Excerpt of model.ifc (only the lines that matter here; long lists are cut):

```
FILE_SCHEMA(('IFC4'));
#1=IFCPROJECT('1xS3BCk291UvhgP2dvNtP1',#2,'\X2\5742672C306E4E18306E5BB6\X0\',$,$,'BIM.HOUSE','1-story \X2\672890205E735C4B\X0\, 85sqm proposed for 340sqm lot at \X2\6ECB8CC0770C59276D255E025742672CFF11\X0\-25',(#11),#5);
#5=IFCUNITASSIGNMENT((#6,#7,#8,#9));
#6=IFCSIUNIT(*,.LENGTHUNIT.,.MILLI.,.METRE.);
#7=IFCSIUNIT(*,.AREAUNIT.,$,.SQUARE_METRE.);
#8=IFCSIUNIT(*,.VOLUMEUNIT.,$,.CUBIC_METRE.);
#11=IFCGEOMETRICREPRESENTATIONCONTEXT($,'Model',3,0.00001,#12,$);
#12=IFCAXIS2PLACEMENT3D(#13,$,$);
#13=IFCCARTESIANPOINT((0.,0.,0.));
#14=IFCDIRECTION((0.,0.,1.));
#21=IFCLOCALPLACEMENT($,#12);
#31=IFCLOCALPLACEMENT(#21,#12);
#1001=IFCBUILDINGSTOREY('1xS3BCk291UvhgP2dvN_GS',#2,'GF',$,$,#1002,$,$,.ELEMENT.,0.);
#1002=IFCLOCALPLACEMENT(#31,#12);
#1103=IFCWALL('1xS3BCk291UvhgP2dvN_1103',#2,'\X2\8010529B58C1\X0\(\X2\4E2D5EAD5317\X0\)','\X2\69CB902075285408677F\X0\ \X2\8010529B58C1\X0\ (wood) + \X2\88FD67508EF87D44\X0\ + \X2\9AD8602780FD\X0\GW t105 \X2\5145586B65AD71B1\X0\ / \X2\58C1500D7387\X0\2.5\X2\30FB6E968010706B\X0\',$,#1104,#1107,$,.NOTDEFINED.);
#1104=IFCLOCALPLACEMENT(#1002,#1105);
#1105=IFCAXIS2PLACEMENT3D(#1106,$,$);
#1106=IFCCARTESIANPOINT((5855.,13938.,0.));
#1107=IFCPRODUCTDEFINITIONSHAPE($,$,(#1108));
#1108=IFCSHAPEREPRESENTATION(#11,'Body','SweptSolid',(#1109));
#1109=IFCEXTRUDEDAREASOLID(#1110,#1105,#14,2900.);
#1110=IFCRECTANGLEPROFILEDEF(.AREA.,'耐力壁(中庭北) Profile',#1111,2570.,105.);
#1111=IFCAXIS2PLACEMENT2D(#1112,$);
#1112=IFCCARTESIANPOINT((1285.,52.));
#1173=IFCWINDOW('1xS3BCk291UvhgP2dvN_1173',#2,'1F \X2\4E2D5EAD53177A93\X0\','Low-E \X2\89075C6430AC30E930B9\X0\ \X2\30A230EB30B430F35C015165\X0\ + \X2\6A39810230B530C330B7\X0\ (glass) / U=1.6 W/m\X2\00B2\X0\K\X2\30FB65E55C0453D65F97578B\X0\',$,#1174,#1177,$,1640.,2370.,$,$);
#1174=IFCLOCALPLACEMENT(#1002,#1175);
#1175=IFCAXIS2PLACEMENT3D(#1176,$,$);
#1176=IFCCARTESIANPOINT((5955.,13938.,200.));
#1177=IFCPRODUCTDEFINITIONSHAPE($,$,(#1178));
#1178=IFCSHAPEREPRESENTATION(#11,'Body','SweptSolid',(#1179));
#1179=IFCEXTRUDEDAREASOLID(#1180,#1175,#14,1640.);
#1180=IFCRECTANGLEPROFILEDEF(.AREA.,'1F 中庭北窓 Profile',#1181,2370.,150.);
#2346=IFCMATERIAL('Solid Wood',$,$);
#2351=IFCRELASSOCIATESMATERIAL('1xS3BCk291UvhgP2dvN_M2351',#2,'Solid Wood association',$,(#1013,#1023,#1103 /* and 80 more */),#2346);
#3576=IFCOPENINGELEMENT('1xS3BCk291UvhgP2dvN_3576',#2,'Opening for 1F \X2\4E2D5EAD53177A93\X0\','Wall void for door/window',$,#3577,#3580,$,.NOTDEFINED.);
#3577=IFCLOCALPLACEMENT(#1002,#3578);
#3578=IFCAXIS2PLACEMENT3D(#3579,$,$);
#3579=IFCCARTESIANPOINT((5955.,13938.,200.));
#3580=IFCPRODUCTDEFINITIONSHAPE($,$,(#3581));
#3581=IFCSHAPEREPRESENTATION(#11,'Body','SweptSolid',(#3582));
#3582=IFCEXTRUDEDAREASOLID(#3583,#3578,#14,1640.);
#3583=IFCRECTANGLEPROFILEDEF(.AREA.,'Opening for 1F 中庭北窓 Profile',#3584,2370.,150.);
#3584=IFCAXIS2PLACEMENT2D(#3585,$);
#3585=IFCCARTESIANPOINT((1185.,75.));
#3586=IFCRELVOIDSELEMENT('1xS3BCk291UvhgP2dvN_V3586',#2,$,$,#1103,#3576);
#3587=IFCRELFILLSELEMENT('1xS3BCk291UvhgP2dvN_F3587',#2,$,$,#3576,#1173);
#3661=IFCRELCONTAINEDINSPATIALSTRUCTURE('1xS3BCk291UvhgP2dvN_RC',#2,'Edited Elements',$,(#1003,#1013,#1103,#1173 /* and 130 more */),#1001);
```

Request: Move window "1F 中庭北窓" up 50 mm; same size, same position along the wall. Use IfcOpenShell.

```python
import numpy as np
import ifcopenshell
import ifcopenshell.api.geometry
import ifcopenshell.util.placement
import ifcopenshell.util.unit

model = ifcopenshell.open("model.ifc")
unit_scale = ifcopenshell.util.unit.calculate_unit_scale(model)

window = model.by_guid("1xS3BCk291UvhgP2dvN_1173")
opening = window.FillsVoids[0].RelatingOpeningElement
dz = 50.0

shift = np.array([0.0, 0.0, dz])
# The window is not placed relative to its opening, so move both.
for product in (opening, window):
    matrix = ifcopenshell.util.placement.get_local_placement(product.ObjectPlacement)
    matrix[:3, 3] += shift
    ifcopenshell.api.geometry.edit_object_placement(model, product=product, matrix=matrix, is_si=False)

print(f"moved by {dz * unit_scale:+.3f} m")

model.write("model-out.ifc")
```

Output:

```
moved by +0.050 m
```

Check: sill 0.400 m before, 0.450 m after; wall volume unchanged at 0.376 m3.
